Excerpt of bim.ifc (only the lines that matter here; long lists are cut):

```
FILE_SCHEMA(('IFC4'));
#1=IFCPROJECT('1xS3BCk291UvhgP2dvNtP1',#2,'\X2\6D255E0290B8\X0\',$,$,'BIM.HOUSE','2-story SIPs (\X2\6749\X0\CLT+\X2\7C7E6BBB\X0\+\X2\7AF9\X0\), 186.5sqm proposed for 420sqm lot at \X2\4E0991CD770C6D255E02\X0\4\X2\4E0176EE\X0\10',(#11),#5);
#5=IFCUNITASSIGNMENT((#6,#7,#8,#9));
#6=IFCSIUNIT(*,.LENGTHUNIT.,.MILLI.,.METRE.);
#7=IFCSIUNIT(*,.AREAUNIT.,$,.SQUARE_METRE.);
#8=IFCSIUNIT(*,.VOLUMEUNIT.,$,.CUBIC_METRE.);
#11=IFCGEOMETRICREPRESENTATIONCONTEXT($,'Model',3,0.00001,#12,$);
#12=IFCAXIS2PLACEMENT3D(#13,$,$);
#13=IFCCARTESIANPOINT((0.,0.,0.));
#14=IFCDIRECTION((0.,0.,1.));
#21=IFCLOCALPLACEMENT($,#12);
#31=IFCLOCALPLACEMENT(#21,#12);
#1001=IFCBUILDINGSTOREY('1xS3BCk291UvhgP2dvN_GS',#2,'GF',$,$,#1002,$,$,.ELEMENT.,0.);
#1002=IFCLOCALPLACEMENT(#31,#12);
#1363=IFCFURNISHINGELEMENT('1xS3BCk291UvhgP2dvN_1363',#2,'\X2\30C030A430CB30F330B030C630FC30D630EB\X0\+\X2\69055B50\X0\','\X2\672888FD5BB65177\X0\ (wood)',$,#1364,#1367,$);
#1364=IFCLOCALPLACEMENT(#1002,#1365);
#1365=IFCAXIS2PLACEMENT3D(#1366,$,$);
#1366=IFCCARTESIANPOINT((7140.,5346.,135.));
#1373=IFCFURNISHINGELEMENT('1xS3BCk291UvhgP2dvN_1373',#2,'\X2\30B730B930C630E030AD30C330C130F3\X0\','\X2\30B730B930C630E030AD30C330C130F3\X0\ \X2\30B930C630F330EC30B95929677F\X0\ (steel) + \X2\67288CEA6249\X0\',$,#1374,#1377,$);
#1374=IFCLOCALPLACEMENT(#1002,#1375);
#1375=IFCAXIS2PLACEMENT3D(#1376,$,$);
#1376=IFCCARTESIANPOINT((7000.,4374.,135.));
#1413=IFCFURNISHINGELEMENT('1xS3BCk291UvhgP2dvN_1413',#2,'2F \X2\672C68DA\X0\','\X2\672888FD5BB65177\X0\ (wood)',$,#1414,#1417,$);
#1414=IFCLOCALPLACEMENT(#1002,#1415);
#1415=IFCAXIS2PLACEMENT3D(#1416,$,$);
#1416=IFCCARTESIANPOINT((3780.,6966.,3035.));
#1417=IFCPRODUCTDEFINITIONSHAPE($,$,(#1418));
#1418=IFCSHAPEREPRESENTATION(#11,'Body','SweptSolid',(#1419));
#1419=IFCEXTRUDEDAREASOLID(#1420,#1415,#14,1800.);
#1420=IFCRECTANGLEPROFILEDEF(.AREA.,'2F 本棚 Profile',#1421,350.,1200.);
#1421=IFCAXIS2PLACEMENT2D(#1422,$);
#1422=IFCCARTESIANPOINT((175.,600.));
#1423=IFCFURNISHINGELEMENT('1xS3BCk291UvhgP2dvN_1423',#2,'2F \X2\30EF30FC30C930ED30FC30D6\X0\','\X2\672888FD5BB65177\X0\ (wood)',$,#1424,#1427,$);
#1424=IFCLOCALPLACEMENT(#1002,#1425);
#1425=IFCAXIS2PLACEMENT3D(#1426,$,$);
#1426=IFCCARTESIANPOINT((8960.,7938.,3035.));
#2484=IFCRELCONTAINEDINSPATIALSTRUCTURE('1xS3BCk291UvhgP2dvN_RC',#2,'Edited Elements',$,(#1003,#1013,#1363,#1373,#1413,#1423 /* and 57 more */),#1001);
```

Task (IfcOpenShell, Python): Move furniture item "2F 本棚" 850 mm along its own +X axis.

```python
import ifcopenshell
import ifcopenshell.api.geometry
import ifcopenshell.util.placement

model = ifcopenshell.open("bim.ifc")

item = model.by_id(1413)
matrix = ifcopenshell.util.placement.get_local_placement(item.ObjectPlacement)
matrix[:3, 3] += matrix[:3, 0] * 850.0
ifcopenshell.api.geometry.edit_object_placement(model, product=item, matrix=matrix, is_si=False)

print(ifcopenshell.util.placement.get_local_placement(item.ObjectPlacement).round(3) + 0.0)

model.write("bim-out.ifc")
```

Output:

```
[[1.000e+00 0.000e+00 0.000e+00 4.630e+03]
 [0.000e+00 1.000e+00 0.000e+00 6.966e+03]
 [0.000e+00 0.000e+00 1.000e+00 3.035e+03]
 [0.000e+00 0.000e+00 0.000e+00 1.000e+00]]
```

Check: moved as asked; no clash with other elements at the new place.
